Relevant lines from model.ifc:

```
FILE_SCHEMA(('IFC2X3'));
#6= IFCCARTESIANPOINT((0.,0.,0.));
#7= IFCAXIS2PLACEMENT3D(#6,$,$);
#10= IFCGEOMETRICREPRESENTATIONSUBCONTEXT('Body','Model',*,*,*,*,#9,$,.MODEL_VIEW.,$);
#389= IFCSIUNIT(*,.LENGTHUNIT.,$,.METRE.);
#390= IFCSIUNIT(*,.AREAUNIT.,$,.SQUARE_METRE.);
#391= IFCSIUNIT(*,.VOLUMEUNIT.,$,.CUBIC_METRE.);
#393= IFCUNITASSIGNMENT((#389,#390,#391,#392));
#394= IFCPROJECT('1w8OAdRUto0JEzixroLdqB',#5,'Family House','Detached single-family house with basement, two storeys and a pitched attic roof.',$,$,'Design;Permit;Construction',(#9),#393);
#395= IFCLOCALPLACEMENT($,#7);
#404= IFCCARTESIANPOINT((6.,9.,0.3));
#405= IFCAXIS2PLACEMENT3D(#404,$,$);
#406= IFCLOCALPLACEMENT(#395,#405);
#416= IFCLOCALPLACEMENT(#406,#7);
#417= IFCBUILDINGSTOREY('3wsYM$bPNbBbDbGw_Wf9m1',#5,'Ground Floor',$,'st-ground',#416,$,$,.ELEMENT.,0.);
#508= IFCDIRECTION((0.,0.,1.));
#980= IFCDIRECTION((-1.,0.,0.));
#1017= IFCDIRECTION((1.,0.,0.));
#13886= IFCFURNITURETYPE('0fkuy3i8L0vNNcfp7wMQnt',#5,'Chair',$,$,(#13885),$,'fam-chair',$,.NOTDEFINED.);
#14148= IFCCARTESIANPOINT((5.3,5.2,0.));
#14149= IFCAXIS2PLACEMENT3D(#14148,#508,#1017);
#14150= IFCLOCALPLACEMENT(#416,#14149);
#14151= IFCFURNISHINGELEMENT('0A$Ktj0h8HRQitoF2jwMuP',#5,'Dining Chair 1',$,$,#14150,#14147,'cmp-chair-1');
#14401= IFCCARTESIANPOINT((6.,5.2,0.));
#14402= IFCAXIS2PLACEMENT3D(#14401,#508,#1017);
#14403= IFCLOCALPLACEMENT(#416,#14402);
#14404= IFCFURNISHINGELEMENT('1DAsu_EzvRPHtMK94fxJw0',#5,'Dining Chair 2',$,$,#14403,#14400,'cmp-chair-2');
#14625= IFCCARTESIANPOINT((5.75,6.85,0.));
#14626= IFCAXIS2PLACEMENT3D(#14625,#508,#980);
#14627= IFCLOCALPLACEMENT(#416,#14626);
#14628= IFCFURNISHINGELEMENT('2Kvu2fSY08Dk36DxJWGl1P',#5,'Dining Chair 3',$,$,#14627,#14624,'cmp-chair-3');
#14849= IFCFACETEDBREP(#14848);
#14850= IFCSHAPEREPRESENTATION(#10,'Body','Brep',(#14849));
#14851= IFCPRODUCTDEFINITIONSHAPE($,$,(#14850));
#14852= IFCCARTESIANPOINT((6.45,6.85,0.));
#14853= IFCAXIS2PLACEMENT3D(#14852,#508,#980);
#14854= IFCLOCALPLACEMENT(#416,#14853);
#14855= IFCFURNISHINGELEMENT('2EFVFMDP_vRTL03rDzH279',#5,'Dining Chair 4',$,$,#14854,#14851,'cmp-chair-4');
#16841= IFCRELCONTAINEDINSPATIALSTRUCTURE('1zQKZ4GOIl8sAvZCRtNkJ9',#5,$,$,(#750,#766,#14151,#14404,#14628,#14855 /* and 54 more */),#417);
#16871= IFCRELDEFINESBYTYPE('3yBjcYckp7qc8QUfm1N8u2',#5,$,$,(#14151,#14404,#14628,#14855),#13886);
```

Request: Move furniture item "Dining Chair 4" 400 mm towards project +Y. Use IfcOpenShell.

```python
import ifcopenshell
import ifcopenshell.api.geometry
import ifcopenshell.util.placement
import ifcopenshell.util.unit

model = ifcopenshell.open("model.ifc")
unit_scale = ifcopenshell.util.unit.calculate_unit_scale(model)

item = model.by_id(14855)
matrix = ifcopenshell.util.placement.get_local_placement(item.ObjectPlacement)
matrix[1, 3] += 0.4 / unit_scale
ifcopenshell.api.geometry.edit_object_placement(model, product=item, matrix=matrix, is_si=False)

print(ifcopenshell.util.placement.get_local_placement(item.ObjectPlacement).round(3) + 0.0)

model.write("model_updated.ifc")
```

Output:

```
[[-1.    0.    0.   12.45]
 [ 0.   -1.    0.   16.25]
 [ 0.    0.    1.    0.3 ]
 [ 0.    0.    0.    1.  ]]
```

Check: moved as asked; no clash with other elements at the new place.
